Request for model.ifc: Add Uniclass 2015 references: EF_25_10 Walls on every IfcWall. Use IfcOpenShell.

First a look at what the model holds.

```python
import ifcopenshell

model = ifcopenshell.open("model.ifc")
print(model.schema)
print("classifications:", [c.Name for c in model.by_type("IfcClassification")])
for ifc_class in ("IfcDoor", "IfcRoof", "IfcStair", "IfcWall", "IfcWindow"):
    print(ifc_class, len(model.by_type(ifc_class)))
```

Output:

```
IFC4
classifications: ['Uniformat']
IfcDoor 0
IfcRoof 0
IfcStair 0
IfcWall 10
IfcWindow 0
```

```python
import ifcopenshell
import ifcopenshell.api.classification

model = ifcopenshell.open("model.ifc")

system = ifcopenshell.api.classification.add_classification(model, classification="Uniclass 2015")

codes = {
    "IfcWall": ("EF_25_10", "Walls"),
}
for ifc_class, (code, name) in codes.items():
    products = model.by_type(ifc_class)
    ifcopenshell.api.classification.add_reference(
        model, products=products, classification=system, identification=code, name=name
    )
    print(code, len(products))

model.write("model_rev.ifc")
```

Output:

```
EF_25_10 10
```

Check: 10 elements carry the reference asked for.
